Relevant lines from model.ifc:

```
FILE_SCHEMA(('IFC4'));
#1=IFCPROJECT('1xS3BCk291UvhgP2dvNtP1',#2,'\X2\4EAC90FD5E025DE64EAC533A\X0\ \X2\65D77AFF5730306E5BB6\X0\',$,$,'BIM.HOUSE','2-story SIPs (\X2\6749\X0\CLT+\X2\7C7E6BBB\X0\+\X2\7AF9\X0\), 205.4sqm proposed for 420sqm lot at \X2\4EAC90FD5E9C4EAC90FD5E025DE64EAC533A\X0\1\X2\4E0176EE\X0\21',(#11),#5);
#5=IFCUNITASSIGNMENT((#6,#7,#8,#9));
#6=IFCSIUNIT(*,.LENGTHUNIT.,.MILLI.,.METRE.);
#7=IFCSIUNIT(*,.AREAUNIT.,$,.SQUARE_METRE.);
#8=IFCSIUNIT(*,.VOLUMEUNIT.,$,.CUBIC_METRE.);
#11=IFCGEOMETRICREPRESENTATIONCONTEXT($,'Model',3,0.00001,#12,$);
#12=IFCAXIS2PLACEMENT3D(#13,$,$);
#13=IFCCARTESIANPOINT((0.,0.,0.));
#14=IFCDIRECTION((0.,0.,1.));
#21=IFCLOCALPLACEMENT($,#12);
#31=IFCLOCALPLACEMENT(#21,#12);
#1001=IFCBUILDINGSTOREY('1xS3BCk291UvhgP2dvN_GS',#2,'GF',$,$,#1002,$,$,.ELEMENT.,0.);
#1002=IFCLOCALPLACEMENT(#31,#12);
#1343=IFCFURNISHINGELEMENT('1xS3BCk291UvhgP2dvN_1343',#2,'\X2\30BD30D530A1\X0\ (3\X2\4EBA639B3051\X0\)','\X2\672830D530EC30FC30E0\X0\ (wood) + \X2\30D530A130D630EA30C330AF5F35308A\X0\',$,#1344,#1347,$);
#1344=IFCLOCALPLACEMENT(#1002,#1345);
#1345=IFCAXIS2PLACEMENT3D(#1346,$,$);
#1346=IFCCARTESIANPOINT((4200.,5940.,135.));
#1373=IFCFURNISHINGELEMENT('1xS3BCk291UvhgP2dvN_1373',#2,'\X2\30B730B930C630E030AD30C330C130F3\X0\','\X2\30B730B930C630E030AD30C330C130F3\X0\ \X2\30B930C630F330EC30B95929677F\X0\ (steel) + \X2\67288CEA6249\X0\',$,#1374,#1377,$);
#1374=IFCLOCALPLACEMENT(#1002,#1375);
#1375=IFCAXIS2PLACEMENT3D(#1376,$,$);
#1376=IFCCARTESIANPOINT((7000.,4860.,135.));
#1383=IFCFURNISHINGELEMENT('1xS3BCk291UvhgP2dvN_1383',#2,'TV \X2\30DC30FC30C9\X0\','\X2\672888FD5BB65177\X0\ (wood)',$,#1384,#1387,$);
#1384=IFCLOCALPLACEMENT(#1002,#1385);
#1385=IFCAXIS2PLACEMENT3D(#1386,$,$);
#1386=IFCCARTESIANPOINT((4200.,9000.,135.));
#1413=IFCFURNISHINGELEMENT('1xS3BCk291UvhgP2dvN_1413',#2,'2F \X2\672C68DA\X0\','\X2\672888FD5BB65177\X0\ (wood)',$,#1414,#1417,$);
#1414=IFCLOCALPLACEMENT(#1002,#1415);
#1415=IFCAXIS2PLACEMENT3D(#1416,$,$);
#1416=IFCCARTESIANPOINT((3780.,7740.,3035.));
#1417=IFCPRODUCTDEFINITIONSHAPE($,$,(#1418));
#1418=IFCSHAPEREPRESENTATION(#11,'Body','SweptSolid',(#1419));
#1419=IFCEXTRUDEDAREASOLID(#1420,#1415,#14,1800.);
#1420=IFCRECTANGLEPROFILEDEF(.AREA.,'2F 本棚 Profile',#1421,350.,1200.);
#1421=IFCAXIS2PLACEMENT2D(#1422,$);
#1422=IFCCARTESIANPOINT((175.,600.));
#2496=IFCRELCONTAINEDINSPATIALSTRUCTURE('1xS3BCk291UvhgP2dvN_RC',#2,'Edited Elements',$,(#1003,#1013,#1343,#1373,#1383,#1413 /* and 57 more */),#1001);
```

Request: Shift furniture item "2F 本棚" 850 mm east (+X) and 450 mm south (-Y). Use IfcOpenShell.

```python
import ifcopenshell
import ifcopenshell.api.geometry
import ifcopenshell.util.placement

model = ifcopenshell.open("model.ifc")

item = model.by_id(1413)
matrix = ifcopenshell.util.placement.get_local_placement(item.ObjectPlacement)
matrix[0, 3] += 850.0
matrix[1, 3] -= 450.0
ifcopenshell.api.geometry.edit_object_placement(model, product=item, matrix=matrix, is_si=False)

print(ifcopenshell.util.placement.get_local_placement(item.ObjectPlacement).round(3) + 0.0)

model.write("model_v2.ifc")
```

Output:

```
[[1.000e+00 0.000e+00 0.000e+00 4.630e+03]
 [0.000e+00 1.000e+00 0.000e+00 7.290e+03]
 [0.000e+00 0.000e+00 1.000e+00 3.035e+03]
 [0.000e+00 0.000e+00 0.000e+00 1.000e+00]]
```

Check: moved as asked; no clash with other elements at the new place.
